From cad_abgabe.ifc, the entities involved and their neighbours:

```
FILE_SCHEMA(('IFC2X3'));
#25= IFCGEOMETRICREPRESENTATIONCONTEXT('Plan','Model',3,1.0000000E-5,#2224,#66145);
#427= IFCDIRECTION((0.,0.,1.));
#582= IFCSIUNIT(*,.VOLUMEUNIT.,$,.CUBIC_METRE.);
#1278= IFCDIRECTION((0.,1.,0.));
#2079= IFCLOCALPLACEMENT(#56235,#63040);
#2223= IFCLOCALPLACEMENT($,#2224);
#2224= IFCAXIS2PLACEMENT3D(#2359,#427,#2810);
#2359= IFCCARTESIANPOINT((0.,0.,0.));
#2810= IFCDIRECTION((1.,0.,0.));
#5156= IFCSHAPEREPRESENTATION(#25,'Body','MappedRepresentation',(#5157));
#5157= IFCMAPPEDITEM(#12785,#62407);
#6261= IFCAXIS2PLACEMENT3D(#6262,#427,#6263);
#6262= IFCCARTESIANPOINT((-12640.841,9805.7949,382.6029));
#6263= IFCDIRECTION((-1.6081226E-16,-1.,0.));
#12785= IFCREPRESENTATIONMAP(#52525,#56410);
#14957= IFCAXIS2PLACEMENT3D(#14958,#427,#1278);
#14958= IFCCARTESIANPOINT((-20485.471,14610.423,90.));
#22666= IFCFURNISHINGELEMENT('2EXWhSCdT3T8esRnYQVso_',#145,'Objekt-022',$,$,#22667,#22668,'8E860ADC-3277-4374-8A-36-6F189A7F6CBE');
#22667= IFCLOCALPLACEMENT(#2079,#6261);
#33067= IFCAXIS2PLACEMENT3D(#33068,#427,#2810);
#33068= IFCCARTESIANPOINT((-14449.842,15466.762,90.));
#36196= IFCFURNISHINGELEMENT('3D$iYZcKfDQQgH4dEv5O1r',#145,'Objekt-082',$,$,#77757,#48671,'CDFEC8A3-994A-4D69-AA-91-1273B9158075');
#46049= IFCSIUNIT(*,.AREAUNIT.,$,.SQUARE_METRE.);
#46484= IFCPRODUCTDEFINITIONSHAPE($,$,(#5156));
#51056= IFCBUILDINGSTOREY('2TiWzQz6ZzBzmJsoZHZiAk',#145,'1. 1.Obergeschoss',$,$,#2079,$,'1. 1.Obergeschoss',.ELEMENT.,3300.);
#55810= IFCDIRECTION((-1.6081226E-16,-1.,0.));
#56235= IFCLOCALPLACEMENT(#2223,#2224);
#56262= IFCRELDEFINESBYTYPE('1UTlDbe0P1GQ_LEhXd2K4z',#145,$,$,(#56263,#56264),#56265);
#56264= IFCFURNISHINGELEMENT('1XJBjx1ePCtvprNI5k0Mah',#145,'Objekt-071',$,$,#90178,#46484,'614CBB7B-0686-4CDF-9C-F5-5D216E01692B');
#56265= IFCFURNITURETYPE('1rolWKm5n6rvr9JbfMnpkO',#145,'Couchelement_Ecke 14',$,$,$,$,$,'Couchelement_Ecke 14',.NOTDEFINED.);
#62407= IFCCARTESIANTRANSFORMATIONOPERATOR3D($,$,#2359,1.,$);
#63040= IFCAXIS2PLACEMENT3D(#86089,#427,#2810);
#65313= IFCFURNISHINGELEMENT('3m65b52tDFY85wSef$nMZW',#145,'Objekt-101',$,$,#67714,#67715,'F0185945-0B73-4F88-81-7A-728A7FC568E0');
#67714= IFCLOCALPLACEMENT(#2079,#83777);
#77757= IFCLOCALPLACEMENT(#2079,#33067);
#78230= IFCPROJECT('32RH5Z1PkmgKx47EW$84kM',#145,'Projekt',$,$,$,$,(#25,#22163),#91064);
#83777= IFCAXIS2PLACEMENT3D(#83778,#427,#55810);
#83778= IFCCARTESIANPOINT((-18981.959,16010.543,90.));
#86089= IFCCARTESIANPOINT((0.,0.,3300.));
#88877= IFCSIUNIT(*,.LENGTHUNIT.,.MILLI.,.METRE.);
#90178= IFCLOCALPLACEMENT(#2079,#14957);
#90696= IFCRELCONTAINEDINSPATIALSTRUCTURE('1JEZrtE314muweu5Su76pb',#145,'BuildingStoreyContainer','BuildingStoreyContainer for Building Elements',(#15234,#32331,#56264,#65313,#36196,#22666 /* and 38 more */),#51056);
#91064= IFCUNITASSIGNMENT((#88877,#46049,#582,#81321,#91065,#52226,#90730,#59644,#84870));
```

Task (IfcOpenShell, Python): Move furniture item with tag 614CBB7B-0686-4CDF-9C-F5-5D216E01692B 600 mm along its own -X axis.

```python
import ifcopenshell
import ifcopenshell.api.geometry
import ifcopenshell.util.placement

model = ifcopenshell.open("cad_abgabe.ifc")

item = model.by_guid("1XJBjx1ePCtvprNI5k0Mah")
matrix = ifcopenshell.util.placement.get_local_placement(item.ObjectPlacement)
matrix[:3, 3] -= matrix[:3, 0] * 600.0
ifcopenshell.api.geometry.edit_object_placement(model, product=item, matrix=matrix, is_si=False)

print(ifcopenshell.util.placement.get_local_placement(item.ObjectPlacement).round(3) + 0.0)

model.write("cad_abgabe-out.ifc")
```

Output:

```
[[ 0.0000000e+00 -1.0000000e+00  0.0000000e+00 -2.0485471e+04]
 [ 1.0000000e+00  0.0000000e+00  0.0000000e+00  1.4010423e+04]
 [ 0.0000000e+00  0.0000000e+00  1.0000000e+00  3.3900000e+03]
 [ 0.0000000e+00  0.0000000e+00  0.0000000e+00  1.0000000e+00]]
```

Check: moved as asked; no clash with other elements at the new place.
